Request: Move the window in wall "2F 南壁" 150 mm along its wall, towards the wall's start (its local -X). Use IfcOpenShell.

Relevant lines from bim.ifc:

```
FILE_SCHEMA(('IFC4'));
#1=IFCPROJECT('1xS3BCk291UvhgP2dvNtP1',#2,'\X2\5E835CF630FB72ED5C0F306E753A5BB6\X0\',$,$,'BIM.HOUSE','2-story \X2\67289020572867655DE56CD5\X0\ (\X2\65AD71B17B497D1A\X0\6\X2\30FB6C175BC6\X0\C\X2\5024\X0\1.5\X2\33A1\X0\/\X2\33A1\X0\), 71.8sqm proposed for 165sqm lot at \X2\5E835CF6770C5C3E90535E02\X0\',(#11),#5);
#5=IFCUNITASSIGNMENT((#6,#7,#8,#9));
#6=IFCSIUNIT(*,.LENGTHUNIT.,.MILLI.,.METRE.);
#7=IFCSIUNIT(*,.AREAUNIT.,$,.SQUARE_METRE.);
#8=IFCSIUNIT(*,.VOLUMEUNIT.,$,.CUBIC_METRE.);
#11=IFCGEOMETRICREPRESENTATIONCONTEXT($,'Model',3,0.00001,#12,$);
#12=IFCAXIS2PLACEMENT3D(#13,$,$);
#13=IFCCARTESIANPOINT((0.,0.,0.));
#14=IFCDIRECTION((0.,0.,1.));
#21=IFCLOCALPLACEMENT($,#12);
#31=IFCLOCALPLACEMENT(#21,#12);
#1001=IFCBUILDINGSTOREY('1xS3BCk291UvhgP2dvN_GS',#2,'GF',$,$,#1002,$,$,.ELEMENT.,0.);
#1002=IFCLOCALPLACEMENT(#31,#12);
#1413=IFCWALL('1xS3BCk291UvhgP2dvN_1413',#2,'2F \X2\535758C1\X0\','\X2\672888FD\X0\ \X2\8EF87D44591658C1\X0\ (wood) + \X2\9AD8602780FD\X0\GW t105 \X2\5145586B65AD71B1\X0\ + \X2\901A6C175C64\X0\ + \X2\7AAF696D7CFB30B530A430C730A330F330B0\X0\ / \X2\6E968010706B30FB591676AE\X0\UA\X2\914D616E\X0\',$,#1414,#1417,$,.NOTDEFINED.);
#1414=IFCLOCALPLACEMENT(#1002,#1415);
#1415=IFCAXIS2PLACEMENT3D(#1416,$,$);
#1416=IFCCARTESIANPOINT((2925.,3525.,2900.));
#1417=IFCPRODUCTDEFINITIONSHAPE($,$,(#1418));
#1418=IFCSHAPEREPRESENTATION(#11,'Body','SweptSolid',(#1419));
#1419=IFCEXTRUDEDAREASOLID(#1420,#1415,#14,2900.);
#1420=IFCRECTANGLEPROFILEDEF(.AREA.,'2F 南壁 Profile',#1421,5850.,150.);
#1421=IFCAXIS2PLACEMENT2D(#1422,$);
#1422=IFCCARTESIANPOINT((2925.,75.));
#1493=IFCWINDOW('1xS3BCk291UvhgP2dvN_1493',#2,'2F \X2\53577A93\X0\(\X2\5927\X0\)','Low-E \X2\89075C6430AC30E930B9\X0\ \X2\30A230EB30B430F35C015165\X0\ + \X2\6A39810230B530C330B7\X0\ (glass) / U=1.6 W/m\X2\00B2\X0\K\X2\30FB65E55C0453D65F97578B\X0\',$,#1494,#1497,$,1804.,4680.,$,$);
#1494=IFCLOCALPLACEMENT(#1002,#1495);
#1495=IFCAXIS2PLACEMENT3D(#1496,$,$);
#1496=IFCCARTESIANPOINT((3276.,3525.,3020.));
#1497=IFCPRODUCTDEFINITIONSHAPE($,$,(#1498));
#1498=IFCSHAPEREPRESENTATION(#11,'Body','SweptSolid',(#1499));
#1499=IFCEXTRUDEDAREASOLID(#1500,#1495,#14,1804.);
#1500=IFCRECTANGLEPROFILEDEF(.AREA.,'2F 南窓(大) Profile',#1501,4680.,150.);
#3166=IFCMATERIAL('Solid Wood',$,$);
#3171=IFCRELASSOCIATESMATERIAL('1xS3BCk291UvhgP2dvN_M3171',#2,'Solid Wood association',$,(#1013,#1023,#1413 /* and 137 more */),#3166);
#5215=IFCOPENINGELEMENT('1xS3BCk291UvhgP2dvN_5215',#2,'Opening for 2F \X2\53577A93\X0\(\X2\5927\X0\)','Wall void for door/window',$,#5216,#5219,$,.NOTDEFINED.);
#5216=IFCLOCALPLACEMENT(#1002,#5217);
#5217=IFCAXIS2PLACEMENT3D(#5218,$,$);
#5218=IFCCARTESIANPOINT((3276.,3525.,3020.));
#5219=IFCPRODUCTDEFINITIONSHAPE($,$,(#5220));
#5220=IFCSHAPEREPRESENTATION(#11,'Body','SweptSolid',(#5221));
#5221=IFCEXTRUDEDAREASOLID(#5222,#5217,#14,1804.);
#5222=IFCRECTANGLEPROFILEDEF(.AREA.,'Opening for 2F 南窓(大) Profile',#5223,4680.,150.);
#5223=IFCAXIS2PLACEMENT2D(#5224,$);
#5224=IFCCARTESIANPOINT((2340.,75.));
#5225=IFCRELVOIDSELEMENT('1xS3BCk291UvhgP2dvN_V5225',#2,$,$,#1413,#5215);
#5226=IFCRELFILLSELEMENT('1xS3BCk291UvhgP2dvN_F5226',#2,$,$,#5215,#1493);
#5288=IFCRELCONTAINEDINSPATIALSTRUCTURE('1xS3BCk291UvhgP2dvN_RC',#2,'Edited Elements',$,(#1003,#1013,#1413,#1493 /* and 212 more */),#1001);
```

```python
import ifcopenshell
import ifcopenshell.api.geometry
import ifcopenshell.util.placement
import ifcopenshell.util.unit

model = ifcopenshell.open("bim.ifc")
unit_scale = ifcopenshell.util.unit.calculate_unit_scale(model)

window = model.by_id(1493)
opening = window.FillsVoids[0].RelatingOpeningElement
wall = opening.VoidsElements[0].RelatingBuildingElement

wall_matrix = ifcopenshell.util.placement.get_local_placement(wall.ObjectPlacement)
shift = wall_matrix[:3, 0] * -0.15 / unit_scale
before = ifcopenshell.util.placement.get_local_placement(window.ObjectPlacement)[:3, 3].copy()

# The window is not placed relative to its opening, so move both.
for product in (opening, window):
    matrix = ifcopenshell.util.placement.get_local_placement(product.ObjectPlacement)
    matrix[:3, 3] += shift
    ifcopenshell.api.geometry.edit_object_placement(model, product=product, matrix=matrix, is_si=False)

after = ifcopenshell.util.placement.get_local_placement(window.ObjectPlacement)[:3, 3]
print("window moved by", (after - before).round(3) + 0.0)

model.write("bim_v2.ifc")
```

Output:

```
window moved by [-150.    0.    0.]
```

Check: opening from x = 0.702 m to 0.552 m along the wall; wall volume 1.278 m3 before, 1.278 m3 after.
